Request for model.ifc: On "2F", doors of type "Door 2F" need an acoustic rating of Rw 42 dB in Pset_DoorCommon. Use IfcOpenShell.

First a look at what the model holds.

```python
import ifcopenshell
import ifcopenshell.util.element

model = ifcopenshell.open("model.ifc")
print(model.schema)
storey = next(s for s in model.by_type("IfcBuildingStorey") if s.Name == "2F")
doors = [e for e in ifcopenshell.util.element.get_decomposition(storey) if e.is_a("IfcDoor")]
seen = {}
for e in doors:
    element_type = ifcopenshell.util.element.get_type(e)
    key = (element_type.Name if element_type != e and element_type else None, ifcopenshell.util.element.get_pset(e, "Pset_DoorCommon", "AcousticRating"))
    seen[key] = seen.get(key, 0) + 1
for (name, value), count in sorted(seen.items(), key=str):
    print(count, "x", name, "|", value)
```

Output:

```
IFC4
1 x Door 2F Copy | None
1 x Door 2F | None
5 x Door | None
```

```python
import ifcopenshell
import ifcopenshell.api.pset
import ifcopenshell.util.element

model = ifcopenshell.open("model.ifc")

storey = next(s for s in model.by_type("IfcBuildingStorey") if s.Name == "2F")
doors = [e for e in ifcopenshell.util.element.get_decomposition(storey) if e.is_a("IfcDoor")]

count = 0
for e in doors:
    element_type = ifcopenshell.util.element.get_type(e)
    if element_type in (None, e) or element_type.Name != "Door 2F":
        continue
    # add_pset returns the element's existing set when there is one.
    pset = ifcopenshell.api.pset.add_pset(model, product=e, name="Pset_DoorCommon")
    ifcopenshell.api.pset.edit_pset(model, pset=pset, properties={"AcousticRating": "Rw 42 dB"})
    count += 1

print(count, "doors updated")

model.write("model_edited.ifc")
```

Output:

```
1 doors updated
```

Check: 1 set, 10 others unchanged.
